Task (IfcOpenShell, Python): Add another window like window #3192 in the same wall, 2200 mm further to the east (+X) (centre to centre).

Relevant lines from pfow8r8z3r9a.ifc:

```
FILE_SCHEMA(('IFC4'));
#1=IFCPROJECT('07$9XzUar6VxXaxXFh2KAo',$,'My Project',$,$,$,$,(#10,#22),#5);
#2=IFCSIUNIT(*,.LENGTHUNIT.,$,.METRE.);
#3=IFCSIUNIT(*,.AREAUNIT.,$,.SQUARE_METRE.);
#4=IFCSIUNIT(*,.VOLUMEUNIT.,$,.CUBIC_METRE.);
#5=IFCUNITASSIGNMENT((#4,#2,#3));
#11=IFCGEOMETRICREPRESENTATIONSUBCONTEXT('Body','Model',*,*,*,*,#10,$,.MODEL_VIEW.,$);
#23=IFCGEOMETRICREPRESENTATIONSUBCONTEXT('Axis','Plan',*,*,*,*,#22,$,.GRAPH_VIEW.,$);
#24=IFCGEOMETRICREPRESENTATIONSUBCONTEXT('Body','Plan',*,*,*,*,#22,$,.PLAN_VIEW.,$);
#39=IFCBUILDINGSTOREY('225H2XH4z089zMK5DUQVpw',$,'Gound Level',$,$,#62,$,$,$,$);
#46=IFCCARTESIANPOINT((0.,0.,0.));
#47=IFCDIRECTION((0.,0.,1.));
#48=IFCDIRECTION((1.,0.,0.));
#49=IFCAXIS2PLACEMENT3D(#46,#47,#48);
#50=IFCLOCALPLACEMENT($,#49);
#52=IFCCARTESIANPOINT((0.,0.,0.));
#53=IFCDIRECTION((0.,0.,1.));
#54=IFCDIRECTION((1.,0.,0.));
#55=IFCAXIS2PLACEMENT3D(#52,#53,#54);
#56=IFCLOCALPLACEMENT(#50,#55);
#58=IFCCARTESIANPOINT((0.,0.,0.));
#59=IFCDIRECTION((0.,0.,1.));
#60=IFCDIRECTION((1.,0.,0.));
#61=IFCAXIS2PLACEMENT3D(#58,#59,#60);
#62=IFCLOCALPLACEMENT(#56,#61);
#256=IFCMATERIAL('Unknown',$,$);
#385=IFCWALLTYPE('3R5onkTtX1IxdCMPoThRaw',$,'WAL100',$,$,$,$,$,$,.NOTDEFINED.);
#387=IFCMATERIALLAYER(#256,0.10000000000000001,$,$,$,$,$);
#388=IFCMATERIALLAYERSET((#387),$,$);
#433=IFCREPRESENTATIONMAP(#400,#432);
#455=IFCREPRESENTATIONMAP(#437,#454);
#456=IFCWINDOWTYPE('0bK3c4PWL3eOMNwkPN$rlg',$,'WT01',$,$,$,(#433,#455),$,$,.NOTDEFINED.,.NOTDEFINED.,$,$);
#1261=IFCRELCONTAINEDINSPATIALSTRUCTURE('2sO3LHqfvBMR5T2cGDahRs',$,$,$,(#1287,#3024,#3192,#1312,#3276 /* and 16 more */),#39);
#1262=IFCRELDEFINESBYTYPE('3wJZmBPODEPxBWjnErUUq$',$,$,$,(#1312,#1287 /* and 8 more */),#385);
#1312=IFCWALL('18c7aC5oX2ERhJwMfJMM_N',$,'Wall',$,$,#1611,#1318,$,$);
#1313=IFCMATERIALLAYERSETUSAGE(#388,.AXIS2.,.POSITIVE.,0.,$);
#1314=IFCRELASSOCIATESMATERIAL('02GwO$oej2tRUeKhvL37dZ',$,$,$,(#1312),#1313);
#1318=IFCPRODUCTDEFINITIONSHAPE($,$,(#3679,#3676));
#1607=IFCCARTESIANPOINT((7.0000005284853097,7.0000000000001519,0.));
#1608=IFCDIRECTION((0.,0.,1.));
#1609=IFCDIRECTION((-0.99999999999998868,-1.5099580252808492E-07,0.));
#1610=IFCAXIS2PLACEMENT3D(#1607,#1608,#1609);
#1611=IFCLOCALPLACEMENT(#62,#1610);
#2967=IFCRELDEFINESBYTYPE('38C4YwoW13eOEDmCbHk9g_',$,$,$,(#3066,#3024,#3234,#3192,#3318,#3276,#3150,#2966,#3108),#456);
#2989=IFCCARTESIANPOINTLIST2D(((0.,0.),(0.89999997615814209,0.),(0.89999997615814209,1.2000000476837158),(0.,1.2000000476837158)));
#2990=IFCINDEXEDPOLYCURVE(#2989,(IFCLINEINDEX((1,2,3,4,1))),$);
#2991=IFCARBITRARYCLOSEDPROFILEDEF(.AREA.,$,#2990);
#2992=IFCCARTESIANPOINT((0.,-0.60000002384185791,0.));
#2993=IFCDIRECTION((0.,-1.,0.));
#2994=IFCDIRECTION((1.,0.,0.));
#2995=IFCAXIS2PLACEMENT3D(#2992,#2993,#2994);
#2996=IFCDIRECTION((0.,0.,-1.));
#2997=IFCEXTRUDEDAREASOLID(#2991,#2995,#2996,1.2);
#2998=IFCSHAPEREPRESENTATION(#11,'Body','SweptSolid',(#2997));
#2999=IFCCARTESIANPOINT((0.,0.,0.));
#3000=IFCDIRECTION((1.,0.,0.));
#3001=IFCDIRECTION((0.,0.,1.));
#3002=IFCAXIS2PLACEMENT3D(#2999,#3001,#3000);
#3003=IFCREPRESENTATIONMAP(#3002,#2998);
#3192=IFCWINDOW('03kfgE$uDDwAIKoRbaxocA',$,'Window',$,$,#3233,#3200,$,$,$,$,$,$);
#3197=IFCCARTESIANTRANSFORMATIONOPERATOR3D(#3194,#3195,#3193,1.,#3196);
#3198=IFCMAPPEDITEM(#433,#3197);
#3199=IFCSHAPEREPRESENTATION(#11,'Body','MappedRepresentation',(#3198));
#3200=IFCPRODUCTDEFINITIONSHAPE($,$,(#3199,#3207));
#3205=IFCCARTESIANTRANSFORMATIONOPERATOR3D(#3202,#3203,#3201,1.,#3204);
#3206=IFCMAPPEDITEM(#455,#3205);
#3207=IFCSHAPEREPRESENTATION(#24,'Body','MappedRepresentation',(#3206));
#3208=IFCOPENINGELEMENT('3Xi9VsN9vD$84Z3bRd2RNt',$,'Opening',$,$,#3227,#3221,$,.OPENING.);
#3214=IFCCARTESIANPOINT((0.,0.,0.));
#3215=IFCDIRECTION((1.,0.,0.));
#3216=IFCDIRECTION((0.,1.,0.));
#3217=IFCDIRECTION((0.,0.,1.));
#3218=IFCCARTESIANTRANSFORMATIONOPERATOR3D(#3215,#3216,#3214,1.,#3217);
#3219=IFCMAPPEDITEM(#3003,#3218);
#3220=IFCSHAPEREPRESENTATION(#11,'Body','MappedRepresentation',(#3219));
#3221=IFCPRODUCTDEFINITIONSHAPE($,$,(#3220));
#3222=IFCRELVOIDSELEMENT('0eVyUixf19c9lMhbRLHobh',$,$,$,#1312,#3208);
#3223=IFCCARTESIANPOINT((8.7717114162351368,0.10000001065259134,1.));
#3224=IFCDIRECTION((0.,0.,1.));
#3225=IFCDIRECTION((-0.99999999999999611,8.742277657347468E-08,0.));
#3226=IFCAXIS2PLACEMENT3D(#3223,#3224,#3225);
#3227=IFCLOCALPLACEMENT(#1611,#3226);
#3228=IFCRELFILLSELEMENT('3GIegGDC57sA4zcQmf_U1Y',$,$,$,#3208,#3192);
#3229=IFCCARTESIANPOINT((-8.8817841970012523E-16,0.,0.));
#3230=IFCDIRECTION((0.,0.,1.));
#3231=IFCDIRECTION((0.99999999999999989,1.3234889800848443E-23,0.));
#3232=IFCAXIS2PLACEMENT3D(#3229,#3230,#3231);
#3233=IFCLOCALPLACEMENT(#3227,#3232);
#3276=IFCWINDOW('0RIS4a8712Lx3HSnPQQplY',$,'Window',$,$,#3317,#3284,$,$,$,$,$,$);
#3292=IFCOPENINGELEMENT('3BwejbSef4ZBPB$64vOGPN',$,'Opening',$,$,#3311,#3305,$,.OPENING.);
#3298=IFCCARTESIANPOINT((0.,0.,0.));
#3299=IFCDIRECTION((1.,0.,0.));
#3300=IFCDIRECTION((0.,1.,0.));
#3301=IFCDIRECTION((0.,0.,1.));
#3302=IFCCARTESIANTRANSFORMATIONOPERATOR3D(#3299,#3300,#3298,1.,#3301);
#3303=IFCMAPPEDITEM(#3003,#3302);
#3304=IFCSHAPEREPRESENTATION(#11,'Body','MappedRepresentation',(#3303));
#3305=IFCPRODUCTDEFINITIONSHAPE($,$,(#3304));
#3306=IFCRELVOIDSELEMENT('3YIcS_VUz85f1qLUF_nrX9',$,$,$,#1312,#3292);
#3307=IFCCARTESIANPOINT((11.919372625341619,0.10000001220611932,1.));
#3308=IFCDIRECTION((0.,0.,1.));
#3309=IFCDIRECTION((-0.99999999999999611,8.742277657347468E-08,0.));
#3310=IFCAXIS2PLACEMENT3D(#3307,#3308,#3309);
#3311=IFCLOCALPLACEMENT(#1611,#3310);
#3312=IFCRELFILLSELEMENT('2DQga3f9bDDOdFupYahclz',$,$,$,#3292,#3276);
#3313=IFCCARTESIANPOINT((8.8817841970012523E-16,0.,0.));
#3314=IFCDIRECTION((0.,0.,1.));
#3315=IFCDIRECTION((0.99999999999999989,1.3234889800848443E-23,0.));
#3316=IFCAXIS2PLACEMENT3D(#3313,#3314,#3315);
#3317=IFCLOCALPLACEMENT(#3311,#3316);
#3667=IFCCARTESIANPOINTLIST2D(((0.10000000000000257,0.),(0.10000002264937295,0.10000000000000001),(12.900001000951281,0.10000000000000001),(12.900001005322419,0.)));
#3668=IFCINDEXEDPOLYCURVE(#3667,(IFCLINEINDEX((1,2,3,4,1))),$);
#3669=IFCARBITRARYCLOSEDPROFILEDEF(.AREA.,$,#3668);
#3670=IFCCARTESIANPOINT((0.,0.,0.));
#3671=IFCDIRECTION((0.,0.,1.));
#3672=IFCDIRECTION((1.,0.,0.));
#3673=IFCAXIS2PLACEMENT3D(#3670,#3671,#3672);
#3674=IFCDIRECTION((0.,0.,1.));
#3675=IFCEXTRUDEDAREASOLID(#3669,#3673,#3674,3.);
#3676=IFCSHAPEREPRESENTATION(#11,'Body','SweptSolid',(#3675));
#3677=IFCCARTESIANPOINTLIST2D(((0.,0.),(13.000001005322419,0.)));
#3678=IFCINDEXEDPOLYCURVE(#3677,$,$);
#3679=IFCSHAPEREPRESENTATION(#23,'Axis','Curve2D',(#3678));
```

```python
import ifcopenshell
import ifcopenshell.api.feature
import ifcopenshell.api.geometry
import ifcopenshell.api.root
import ifcopenshell.geom
import ifcopenshell.util.element
import ifcopenshell.util.placement
import ifcopenshell.util.shape
import ifcopenshell.util.unit

model = ifcopenshell.open("pfow8r8z3r9a.ifc")
unit_scale = ifcopenshell.util.unit.calculate_unit_scale(model)
settings = ifcopenshell.geom.settings()


def volume(element):
    """Net volume in cubic metres, openings subtracted."""
    shape = ifcopenshell.geom.create_shape(settings, element)
    return ifcopenshell.util.shape.get_volume(shape.geometry)


window = model.by_guid("03kfgE$uDDwAIKoRbaxocA")
opening = window.FillsVoids[0].RelatingOpeningElement
wall = opening.VoidsElements[0].RelatingBuildingElement
before = volume(wall)
shift = ifcopenshell.util.placement.get_local_placement(wall.ObjectPlacement)[:3, 0] * -2.2 / unit_scale

# copy_class copies the void relationship, type, container and properties, but no geometry.
new_opening = ifcopenshell.api.root.copy_class(model, product=opening)
new_opening.Representation = ifcopenshell.util.element.copy_deep(
    model, opening.Representation, exclude=["IfcGeometricRepresentationContext", "IfcRepresentationMap"]
)
new_window = ifcopenshell.api.root.copy_class(model, product=window)
new_window.Representation = ifcopenshell.util.element.copy_deep(
    model, window.Representation, exclude=["IfcGeometricRepresentationContext", "IfcRepresentationMap"]
)
ifcopenshell.api.feature.add_filling(model, opening=new_opening, element=new_window)

for old, new in ((opening, new_opening), (window, new_window)):
    matrix = ifcopenshell.util.placement.get_local_placement(old.ObjectPlacement)
    matrix[:3, 3] += shift
    ifcopenshell.api.geometry.edit_object_placement(model, product=new, matrix=matrix, is_si=False)

after = volume(wall)

print(f"wall volume {before:.3f} -> {after:.3f} m3")

model.write("pfow8r8z3r9a_v2.ifc")
```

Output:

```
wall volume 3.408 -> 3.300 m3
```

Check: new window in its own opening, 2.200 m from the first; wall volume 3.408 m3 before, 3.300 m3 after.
